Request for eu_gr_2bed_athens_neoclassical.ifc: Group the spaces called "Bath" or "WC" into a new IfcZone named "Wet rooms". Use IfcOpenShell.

First a look at what the model holds.

```python
import ifcopenshell

model = ifcopenshell.open("eu_gr_2bed_athens_neoclassical.ifc")
print(model.schema)
seen = {}
for space in model.by_type("IfcSpace"):
    seen[space.LongName] = seen.get(space.LongName, 0) + 1
for name, count in sorted(seen.items(), key=str):
    print(count, "x", name)
print("zones:", [z.Name for z in model.by_type("IfcZone")][:20])
```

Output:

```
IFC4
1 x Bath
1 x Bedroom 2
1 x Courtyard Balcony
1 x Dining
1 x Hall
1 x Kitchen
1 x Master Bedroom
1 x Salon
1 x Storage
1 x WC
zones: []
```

```python
import ifcopenshell
import ifcopenshell.api.group
import ifcopenshell.api.root

model = ifcopenshell.open("eu_gr_2bed_athens_neoclassical.ifc")

names = {"Bath", "WC"}
spaces = [s for s in model.by_type("IfcSpace") if s.LongName in names]

zone = ifcopenshell.api.root.create_entity(model, ifc_class="IfcZone", name="Wet rooms")
ifcopenshell.api.group.assign_group(model, products=spaces, group=zone)
print(len(spaces), "spaces in", zone.Name)

model.write("eu_gr_2bed_athens_neoclassical_edited.ifc")
```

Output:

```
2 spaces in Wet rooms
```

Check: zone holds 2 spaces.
